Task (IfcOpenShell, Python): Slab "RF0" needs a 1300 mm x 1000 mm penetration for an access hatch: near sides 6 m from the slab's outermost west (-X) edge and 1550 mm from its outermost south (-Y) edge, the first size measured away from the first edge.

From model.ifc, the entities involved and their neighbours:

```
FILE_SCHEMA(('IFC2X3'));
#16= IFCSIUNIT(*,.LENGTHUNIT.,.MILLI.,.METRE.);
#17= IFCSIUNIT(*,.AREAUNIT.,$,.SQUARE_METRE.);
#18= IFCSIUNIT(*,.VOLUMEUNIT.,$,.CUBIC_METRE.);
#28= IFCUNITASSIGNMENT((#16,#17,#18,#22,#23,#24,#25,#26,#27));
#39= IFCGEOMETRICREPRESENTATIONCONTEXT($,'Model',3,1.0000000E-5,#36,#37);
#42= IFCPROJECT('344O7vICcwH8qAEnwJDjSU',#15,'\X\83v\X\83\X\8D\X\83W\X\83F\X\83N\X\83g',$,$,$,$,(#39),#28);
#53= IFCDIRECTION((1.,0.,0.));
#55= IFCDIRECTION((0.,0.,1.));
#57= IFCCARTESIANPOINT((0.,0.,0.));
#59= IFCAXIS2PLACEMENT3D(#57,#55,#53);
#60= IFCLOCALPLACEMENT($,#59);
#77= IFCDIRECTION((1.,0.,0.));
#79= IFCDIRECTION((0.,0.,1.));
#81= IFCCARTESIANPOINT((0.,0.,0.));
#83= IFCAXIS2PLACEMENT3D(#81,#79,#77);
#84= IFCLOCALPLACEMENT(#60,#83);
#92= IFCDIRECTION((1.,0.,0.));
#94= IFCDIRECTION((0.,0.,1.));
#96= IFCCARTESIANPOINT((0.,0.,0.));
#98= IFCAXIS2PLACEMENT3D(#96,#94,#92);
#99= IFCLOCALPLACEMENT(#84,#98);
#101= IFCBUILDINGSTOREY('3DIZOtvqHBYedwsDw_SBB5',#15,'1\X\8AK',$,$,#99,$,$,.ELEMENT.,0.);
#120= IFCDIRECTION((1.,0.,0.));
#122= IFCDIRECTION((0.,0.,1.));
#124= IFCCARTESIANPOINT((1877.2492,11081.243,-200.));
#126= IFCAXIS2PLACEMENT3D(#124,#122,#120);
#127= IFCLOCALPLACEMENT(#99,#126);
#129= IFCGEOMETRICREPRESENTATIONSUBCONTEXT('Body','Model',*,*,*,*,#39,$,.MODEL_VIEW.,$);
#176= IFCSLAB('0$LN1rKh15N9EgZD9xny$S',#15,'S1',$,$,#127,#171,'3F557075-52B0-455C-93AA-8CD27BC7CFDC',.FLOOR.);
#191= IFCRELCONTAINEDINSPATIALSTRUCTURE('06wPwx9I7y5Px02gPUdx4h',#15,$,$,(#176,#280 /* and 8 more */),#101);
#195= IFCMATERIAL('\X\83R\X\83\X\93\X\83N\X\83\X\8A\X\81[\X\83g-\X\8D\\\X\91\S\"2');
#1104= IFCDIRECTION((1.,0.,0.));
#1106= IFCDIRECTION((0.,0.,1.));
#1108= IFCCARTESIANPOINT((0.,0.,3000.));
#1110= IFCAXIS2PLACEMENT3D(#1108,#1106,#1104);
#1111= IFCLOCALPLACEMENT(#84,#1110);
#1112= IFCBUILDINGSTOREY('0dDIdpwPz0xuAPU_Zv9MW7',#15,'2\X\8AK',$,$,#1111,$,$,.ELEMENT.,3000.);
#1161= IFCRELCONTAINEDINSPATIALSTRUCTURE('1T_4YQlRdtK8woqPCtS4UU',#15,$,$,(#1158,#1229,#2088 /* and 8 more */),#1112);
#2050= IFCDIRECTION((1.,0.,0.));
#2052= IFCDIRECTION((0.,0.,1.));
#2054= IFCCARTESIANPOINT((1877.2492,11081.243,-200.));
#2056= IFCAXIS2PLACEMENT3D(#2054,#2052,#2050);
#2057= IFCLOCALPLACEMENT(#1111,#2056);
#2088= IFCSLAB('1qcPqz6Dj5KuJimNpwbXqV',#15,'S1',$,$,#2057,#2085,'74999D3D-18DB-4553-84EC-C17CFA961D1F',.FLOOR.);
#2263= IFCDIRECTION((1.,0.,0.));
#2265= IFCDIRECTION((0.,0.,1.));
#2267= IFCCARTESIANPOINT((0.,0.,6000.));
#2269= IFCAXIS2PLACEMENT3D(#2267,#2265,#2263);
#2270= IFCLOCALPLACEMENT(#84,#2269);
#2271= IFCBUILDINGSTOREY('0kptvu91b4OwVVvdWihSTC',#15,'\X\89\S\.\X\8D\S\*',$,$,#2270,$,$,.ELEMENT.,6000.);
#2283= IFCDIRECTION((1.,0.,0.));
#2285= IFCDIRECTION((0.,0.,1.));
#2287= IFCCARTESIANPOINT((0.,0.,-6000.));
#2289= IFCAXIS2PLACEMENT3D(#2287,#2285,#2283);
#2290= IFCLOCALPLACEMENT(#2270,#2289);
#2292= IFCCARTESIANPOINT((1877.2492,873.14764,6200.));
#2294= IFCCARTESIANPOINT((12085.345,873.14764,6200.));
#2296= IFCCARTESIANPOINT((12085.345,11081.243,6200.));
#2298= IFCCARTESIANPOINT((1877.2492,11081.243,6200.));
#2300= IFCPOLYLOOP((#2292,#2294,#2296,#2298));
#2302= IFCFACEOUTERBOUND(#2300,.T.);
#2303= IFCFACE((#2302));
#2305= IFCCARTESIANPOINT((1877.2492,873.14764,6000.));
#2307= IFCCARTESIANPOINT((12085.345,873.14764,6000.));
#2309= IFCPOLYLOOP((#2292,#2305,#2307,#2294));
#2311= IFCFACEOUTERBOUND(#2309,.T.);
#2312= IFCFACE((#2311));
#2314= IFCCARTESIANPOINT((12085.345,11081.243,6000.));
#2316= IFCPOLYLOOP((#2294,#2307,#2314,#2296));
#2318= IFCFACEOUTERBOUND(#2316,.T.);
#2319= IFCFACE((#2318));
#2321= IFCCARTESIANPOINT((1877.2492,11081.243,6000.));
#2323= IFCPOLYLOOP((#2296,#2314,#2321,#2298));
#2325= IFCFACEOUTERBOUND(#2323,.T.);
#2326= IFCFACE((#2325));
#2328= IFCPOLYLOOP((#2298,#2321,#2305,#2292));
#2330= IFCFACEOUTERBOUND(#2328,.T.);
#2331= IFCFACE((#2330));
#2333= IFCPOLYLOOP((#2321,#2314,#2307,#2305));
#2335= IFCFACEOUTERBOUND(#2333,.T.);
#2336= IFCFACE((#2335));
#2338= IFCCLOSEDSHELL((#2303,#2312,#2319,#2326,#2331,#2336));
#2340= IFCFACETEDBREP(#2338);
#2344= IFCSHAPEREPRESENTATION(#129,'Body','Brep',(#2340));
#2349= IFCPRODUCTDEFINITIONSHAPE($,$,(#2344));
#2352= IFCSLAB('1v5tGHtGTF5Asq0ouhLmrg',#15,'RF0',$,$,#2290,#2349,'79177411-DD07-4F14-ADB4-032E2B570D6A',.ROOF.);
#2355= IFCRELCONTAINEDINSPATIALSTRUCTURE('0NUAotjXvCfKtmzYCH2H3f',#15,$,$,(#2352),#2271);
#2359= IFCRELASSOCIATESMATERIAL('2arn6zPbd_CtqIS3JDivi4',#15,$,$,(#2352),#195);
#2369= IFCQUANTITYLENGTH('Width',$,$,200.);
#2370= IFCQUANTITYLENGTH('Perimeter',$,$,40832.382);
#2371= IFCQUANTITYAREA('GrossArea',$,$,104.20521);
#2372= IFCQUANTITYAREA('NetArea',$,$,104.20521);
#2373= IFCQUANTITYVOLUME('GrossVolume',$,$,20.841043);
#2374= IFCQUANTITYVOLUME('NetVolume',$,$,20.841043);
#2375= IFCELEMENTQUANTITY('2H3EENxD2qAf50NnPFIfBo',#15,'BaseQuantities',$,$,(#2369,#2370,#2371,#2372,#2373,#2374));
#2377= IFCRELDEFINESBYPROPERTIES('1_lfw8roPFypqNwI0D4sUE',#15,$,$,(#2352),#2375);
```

```python
import numpy as np
import ifcopenshell
import ifcopenshell.api.feature
import ifcopenshell.api.geometry
import ifcopenshell.api.pset
import ifcopenshell.api.root
import ifcopenshell.geom
import ifcopenshell.util.element
import ifcopenshell.util.placement
import ifcopenshell.util.representation
import ifcopenshell.util.shape
import ifcopenshell.util.unit

model = ifcopenshell.open("model.ifc")
unit_scale = ifcopenshell.util.unit.calculate_unit_scale(model)
area_scale = ifcopenshell.util.unit.calculate_unit_scale(model, "AREAUNIT")
volume_scale = ifcopenshell.util.unit.calculate_unit_scale(model, "VOLUMEUNIT")
settings = ifcopenshell.geom.settings()


def volume(element):
    """Net volume in cubic metres, openings subtracted."""
    shape = ifcopenshell.geom.create_shape(settings, element)
    return ifcopenshell.util.shape.get_volume(shape.geometry)


slab = model.by_guid("1v5tGHtGTF5Asq0ouhLmrg")
before = volume(slab)

# Extent in the slab's own axes, in metres. The edges named are its -X and -Y sides.
slab_shape = ifcopenshell.geom.create_shape(settings, slab)
vertices = ifcopenshell.util.shape.get_vertices(slab_shape.geometry)
x_min, y_min, bottom = vertices.min(axis=0)
top = vertices[:, 2].max()

opening = ifcopenshell.api.root.create_entity(model, ifc_class="IfcOpeningElement", name="Access hatch opening")
context = ifcopenshell.util.representation.get_context(model, "Model", "Body", "MODEL_VIEW")
width, depth = 1.3, 1
outline = [(0.0, 0.0), (width, 0.0), (width, depth), (0.0, depth), (0.0, 0.0)]
# Overshoot both faces by 50 mm so the cut is clean.
shape = ifcopenshell.api.geometry.add_slab_representation(
    model, context=context, depth=top - bottom + 0.1, polyline=outline
)
ifcopenshell.api.geometry.assign_representation(model, product=opening, representation=shape)

matrix = ifcopenshell.util.placement.get_local_placement(slab.ObjectPlacement)
matrix[:, 3] = matrix @ np.append(np.array([x_min + 6, y_min + 1.55, bottom - 0.05]) / unit_scale, 1.0)
ifcopenshell.api.geometry.edit_object_placement(model, product=opening, matrix=matrix, is_si=False)
ifcopenshell.api.feature.add_feature(model, feature=opening, element=slab)

after = volume(slab)

# Update the slab's stored quantities.
qto = model.by_id(ifcopenshell.util.element.get_pset(slab, "BaseQuantities", should_inherit=False)["id"])
ifcopenshell.api.pset.edit_qto(model, qto=qto, properties={
    "NetArea": after / (top - bottom) / area_scale,
    "NetVolume": after / volume_scale,
})

print(f"slab volume {before:.3f} -> {after:.3f} m3")

model.write("model_edited.ifc")
```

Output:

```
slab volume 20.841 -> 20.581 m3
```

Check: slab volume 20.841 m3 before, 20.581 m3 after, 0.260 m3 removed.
